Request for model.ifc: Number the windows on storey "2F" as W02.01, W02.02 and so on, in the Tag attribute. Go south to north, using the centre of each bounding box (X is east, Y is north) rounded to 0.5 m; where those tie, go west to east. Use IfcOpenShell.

First a look at what the model holds.

```python
import ifcopenshell
import ifcopenshell.util.element
import ifcopenshell.util.placement

model = ifcopenshell.open("model.ifc")
print(model.schema)
storey = next(s for s in model.by_type("IfcBuildingStorey") if s.Name == "2F")
windows = [e for e in ifcopenshell.util.element.get_decomposition(storey) if e.is_a("IfcWindow")]
for e in sorted(windows, key=lambda e: e.id()):
    origin = ifcopenshell.util.placement.get_local_placement(e.ObjectPlacement)[:3, 3]
    print(e.id(), e.Tag, e.Name, origin.round(2) + 0.0, sep=" | ")
```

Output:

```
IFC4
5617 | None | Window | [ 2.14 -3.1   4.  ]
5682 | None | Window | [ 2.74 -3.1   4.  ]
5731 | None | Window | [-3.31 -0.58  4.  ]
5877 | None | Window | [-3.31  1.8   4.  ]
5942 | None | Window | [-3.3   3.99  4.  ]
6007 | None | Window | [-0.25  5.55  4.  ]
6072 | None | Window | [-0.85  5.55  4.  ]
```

```python
import ifcopenshell
import ifcopenshell.geom
import ifcopenshell.util.element
import ifcopenshell.util.shape

model = ifcopenshell.open("model.ifc")
settings = ifcopenshell.geom.settings()
settings.set("use-world-coords", True)


def centre(element):
    shape = ifcopenshell.geom.create_shape(settings, element)
    return ifcopenshell.util.shape.get_bbox_centroid(shape.geometry)


storey = next(s for s in model.by_type("IfcBuildingStorey") if s.Name == "2F")
windows = [e for e in ifcopenshell.util.element.get_decomposition(storey) if e.is_a("IfcWindow")]

# Insertion points can sit at a corner or the storey origin, so sort by the geometry (in metres).
centres = {e: centre(e) for e in windows}
windows.sort(key=lambda e: (round(centres[e][1] / 0.5), centres[e][0]))

for i, e in enumerate(windows, start=1):
    number = f"W02.{i:02d}"
    e.Tag = number
    print(e.id(), number)

model.write("model_updated.ifc")
```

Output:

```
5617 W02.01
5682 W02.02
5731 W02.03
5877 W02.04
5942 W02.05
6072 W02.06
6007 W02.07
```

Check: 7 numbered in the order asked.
